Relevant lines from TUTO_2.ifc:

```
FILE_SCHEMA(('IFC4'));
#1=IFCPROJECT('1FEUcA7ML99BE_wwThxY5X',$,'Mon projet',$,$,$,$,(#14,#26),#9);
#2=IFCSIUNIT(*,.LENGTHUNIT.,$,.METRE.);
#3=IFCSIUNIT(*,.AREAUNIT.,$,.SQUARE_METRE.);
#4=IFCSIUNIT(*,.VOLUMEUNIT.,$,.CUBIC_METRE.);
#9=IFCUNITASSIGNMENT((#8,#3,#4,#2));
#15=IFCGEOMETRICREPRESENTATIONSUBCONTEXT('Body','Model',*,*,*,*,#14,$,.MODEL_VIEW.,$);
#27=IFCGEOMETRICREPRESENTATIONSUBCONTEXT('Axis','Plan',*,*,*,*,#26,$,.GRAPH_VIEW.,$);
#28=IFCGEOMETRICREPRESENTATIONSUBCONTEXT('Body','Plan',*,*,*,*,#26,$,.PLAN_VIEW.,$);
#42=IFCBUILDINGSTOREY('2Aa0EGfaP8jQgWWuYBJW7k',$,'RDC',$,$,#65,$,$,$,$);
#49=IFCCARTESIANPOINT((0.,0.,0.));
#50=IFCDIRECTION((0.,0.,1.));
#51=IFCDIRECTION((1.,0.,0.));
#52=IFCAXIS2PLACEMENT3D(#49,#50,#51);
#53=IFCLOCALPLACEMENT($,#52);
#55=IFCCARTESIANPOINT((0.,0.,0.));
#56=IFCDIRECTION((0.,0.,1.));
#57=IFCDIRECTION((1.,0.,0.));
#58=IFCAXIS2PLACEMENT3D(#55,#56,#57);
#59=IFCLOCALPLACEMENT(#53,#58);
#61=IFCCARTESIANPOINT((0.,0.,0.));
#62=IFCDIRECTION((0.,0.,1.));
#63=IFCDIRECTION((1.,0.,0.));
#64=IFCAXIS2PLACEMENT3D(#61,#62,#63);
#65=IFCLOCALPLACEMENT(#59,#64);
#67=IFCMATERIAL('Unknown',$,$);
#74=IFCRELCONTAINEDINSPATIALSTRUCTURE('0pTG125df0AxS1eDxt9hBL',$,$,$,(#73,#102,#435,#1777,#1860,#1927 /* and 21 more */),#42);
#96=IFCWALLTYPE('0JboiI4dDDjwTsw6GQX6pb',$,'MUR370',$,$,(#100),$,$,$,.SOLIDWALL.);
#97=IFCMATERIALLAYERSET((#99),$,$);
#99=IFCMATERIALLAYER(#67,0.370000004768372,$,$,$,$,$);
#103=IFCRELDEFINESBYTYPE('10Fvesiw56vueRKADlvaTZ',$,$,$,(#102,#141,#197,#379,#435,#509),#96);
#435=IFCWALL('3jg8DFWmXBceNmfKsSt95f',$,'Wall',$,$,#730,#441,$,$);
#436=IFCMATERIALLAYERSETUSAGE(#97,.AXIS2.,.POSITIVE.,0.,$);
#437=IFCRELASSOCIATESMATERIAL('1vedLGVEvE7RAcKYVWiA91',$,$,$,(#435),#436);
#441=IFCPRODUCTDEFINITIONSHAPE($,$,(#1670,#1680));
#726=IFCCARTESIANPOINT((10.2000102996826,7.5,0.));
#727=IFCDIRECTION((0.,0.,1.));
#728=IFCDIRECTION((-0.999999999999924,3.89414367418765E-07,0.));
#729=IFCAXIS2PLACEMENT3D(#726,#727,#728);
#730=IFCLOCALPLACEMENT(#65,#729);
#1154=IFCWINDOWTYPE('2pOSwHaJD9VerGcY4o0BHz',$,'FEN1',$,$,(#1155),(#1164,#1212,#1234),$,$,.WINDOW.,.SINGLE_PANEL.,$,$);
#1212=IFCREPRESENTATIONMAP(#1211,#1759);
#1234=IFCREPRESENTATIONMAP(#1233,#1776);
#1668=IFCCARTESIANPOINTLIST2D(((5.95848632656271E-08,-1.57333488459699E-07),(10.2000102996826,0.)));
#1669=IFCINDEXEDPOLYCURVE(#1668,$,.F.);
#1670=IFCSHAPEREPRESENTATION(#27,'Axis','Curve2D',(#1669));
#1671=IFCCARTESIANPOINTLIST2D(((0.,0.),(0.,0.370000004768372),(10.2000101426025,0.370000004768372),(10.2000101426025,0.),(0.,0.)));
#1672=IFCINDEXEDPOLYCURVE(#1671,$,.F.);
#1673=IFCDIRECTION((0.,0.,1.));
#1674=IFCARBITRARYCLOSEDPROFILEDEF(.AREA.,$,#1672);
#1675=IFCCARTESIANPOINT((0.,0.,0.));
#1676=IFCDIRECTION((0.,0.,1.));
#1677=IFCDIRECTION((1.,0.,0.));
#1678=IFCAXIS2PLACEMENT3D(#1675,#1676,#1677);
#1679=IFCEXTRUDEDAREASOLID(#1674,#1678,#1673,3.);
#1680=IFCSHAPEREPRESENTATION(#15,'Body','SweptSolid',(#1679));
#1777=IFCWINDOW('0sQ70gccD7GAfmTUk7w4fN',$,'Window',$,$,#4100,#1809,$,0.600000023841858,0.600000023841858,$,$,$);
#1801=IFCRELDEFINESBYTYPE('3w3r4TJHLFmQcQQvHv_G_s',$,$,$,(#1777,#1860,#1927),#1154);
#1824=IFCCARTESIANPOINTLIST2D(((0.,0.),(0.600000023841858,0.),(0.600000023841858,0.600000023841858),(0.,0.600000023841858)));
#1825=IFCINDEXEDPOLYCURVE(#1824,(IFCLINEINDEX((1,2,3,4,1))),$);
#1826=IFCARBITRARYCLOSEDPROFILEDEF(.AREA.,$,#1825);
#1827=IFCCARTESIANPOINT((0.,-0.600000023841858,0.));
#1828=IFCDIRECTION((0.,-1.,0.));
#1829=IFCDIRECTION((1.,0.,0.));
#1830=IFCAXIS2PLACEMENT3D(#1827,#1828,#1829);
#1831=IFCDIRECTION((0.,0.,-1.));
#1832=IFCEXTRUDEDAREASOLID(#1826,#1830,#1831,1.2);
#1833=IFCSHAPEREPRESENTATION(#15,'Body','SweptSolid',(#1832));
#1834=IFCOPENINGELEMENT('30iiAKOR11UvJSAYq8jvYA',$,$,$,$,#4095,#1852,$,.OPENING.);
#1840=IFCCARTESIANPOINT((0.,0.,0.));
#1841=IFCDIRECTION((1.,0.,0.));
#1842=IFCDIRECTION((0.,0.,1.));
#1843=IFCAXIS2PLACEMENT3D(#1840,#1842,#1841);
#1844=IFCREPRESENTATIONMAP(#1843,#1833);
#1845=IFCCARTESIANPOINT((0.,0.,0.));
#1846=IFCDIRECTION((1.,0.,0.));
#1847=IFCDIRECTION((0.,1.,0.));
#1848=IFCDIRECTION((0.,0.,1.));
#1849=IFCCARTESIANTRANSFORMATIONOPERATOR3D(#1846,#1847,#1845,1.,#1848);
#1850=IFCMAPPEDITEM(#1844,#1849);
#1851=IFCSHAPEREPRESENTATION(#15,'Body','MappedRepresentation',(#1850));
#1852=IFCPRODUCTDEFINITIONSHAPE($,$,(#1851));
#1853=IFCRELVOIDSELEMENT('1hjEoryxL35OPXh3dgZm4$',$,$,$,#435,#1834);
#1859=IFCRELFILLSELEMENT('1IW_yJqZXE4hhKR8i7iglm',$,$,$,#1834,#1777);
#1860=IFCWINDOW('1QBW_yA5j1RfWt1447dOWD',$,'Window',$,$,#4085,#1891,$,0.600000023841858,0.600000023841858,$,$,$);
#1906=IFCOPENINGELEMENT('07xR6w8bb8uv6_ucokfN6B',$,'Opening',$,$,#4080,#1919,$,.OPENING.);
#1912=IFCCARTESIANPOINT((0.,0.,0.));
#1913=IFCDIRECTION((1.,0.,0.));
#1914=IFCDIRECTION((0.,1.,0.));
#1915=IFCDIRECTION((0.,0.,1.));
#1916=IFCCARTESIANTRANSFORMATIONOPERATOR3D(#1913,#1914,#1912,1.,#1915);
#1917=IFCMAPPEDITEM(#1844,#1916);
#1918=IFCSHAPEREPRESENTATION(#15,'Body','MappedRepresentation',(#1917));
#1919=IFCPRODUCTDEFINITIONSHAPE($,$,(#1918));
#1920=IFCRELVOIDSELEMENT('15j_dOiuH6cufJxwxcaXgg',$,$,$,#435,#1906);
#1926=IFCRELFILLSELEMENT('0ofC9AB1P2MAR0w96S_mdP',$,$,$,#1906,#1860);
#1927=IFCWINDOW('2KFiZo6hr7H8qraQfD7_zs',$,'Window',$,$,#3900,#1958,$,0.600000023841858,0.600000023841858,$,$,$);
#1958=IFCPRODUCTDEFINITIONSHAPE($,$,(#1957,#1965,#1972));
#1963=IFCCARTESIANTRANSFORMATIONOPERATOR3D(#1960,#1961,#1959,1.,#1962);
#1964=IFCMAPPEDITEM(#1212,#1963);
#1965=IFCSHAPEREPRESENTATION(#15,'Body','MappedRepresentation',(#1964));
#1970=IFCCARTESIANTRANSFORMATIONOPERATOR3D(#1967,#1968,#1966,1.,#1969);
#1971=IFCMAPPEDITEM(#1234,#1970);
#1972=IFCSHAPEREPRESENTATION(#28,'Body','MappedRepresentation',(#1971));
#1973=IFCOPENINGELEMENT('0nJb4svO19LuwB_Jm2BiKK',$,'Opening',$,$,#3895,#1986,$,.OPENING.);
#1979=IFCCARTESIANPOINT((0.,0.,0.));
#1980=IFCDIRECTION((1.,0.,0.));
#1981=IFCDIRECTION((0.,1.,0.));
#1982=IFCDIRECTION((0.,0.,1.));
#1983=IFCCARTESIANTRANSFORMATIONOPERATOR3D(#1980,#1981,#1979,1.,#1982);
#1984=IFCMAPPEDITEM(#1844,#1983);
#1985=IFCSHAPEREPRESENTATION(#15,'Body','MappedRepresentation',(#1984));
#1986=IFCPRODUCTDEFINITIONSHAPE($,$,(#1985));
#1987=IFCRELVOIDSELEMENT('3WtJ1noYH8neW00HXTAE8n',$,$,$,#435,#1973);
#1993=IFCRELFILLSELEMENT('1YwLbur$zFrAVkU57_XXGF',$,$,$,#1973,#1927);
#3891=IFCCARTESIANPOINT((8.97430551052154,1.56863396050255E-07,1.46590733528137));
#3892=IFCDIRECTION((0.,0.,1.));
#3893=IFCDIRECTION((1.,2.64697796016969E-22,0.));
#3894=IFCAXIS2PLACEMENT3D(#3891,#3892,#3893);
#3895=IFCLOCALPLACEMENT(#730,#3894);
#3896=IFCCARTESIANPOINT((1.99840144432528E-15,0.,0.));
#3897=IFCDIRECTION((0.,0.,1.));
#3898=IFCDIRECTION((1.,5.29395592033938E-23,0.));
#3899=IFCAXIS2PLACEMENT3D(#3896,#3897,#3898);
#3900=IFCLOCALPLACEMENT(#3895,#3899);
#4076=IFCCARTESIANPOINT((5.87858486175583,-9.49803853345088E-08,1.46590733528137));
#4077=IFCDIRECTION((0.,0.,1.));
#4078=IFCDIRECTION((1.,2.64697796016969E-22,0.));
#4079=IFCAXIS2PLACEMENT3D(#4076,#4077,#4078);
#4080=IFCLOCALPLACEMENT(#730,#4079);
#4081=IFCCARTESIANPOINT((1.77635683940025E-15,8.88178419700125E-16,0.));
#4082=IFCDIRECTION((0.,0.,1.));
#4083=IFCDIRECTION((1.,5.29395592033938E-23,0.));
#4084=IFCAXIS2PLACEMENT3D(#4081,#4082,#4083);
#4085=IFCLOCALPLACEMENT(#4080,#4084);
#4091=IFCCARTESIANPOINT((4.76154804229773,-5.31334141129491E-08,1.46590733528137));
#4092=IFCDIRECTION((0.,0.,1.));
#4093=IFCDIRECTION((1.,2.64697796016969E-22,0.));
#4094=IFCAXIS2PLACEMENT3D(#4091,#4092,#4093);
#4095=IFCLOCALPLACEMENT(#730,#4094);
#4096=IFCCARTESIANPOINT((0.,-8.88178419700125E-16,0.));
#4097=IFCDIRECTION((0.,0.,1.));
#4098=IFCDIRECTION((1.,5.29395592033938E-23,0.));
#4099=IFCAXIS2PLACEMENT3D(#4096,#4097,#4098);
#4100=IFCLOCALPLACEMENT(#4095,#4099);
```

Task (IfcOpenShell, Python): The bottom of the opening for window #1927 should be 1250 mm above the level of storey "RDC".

```python
import numpy as np
import ifcopenshell
import ifcopenshell.api.geometry
import ifcopenshell.geom
import ifcopenshell.util.element
import ifcopenshell.util.placement
import ifcopenshell.util.shape
import ifcopenshell.util.unit

model = ifcopenshell.open("TUTO_2.ifc")
unit_scale = ifcopenshell.util.unit.calculate_unit_scale(model)

window = model.by_guid("2KFiZo6hr7H8qraQfD7_zs")
opening = window.FillsVoids[0].RelatingOpeningElement
storey = ifcopenshell.util.element.get_container(window, ifc_class="IfcBuildingStorey")
level = ifcopenshell.util.placement.get_local_placement(storey.ObjectPlacement)[2, 3]

# The opening's origin need not be at the sill, so measure its lowest point.
shape = ifcopenshell.geom.create_shape(ifcopenshell.geom.settings(), opening)
bottom = ifcopenshell.util.shape.get_shape_bottom_elevation(shape, shape.geometry) / unit_scale
dz = level + 1.25 - bottom

shift = np.array([0.0, 0.0, dz])
# The window is placed relative to its opening, so it follows when the opening moves.
matrix = ifcopenshell.util.placement.get_local_placement(opening.ObjectPlacement)
matrix[:3, 3] += shift
ifcopenshell.api.geometry.edit_object_placement(
    model, product=opening, matrix=matrix, is_si=False, should_transform_children=True
)

print(f"moved by {dz * unit_scale:+.3f} m")

model.write("TUTO_2_edited.ifc")
```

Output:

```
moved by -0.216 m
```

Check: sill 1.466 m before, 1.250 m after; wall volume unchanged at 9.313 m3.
